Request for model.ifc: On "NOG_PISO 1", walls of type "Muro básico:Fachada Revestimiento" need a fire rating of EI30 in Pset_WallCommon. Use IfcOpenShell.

First a look at what the model holds.

```python
import ifcopenshell
import ifcopenshell.util.element

model = ifcopenshell.open("model.ifc")
print(model.schema)
storey = next(s for s in model.by_type("IfcBuildingStorey") if s.Name == "NOG_PISO 1")
walls = [e for e in ifcopenshell.util.element.get_decomposition(storey) if e.is_a("IfcWall")]
seen = {}
for e in walls:
    element_type = ifcopenshell.util.element.get_type(e)
    key = (element_type.Name if element_type != e and element_type else None, ifcopenshell.util.element.get_pset(e, "Pset_WallCommon", "FireRating"))
    seen[key] = seen.get(key, 0) + 1
for (name, value), count in sorted(seen.items(), key=str):
    print(count, "x", name, "|", value)
```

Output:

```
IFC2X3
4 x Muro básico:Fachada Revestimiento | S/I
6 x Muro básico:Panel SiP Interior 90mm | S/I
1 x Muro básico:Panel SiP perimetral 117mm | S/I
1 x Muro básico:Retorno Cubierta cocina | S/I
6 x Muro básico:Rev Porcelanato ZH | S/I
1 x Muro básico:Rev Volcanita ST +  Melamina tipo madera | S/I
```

```python
import ifcopenshell
import ifcopenshell.api.pset
import ifcopenshell.util.element

model = ifcopenshell.open("model.ifc")

storey = next(s for s in model.by_type("IfcBuildingStorey") if s.Name == "NOG_PISO 1")
walls = [e for e in ifcopenshell.util.element.get_decomposition(storey) if e.is_a("IfcWall")]

count = 0
for e in walls:
    element_type = ifcopenshell.util.element.get_type(e)
    if element_type in (None, e) or element_type.Name != "Muro básico:Fachada Revestimiento":
        continue
    # add_pset returns the element's existing set when there is one.
    pset = ifcopenshell.api.pset.add_pset(model, product=e, name="Pset_WallCommon")
    ifcopenshell.api.pset.edit_pset(model, pset=pset, properties={"FireRating": "EI30"})
    count += 1

print(count, "walls updated")

model.write("model-out.ifc")
```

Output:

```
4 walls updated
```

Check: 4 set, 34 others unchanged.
